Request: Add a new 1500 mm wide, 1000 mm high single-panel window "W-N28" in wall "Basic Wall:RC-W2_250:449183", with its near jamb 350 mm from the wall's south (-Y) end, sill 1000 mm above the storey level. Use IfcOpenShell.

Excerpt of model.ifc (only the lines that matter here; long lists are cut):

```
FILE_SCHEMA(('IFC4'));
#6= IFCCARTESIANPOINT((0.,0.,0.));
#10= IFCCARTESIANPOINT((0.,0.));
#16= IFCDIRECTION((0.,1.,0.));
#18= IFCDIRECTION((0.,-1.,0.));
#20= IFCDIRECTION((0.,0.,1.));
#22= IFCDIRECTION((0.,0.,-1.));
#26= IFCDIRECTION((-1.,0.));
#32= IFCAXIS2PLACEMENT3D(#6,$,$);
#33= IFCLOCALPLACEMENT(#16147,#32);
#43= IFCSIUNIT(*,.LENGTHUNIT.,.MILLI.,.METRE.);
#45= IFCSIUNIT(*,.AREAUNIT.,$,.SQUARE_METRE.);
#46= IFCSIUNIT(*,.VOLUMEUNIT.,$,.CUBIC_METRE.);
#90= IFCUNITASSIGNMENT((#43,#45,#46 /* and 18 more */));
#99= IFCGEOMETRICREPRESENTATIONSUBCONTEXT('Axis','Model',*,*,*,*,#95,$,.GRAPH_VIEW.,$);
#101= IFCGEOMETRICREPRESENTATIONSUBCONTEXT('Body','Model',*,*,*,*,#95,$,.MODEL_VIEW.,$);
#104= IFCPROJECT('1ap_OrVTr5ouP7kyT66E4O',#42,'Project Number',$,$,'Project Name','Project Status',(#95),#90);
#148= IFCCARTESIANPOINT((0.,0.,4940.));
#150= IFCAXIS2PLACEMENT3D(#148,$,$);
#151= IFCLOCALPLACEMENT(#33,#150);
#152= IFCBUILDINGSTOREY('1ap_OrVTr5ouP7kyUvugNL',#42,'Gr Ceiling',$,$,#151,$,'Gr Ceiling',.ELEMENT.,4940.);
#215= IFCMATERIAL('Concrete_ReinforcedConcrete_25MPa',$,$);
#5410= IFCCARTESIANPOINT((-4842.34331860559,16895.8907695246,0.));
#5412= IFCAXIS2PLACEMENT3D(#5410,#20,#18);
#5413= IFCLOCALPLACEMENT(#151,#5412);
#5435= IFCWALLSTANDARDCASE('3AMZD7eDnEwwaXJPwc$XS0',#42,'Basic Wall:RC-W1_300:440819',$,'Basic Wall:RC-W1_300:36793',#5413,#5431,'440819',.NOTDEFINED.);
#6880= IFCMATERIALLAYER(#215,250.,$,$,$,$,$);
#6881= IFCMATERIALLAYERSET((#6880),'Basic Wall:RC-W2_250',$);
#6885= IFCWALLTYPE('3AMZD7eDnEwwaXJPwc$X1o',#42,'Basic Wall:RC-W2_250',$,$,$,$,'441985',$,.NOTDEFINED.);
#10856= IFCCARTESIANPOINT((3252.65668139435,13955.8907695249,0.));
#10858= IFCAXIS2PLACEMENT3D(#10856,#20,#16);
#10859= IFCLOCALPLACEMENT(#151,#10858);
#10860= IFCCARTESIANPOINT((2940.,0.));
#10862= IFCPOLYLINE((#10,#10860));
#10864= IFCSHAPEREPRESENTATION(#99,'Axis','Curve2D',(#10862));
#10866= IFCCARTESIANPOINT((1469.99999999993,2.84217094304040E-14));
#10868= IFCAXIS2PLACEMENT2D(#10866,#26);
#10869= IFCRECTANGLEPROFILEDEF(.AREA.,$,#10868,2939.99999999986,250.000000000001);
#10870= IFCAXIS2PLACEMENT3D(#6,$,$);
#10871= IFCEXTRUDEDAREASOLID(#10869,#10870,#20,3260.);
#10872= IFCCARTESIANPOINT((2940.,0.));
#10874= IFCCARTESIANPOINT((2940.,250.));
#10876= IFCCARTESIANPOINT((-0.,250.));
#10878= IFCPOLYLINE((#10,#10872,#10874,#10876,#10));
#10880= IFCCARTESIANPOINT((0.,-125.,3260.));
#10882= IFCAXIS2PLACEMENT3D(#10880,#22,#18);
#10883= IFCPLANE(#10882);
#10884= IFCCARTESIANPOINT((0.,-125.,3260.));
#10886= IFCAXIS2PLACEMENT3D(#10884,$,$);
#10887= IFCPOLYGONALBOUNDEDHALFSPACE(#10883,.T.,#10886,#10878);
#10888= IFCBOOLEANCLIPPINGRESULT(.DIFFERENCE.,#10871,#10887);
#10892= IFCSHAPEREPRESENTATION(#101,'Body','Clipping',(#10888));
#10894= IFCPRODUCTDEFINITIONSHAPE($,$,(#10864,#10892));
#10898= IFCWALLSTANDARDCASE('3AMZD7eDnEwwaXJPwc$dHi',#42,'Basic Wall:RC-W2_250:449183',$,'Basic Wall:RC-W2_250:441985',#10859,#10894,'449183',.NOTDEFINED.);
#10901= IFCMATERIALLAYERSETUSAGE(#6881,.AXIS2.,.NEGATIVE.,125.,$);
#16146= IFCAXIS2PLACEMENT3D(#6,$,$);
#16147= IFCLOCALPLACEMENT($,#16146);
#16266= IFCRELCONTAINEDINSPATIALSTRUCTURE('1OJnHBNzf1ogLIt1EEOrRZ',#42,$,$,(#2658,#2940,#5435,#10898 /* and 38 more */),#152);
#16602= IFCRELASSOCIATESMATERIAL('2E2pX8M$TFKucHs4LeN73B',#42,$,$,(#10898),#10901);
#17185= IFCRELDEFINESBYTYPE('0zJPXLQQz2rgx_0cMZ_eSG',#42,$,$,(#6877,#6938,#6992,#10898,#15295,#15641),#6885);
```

```python
import numpy as np
import ifcopenshell
import ifcopenshell.api.feature
import ifcopenshell.api.geometry
import ifcopenshell.api.root
import ifcopenshell.api.spatial
import ifcopenshell.geom
import ifcopenshell.util.element
import ifcopenshell.util.placement
import ifcopenshell.util.representation
import ifcopenshell.util.shape
import ifcopenshell.util.unit

model = ifcopenshell.open("model.ifc")
unit_scale = ifcopenshell.util.unit.calculate_unit_scale(model)
settings = ifcopenshell.geom.settings()


def volume(element):
    """Net volume in cubic metres, openings subtracted."""
    shape = ifcopenshell.geom.create_shape(settings, element)
    return ifcopenshell.util.shape.get_volume(shape.geometry)


wall = model.by_guid("3AMZD7eDnEwwaXJPwc$dHi")
storey = ifcopenshell.util.element.get_container(wall, ifc_class="IfcBuildingStorey")
context = ifcopenshell.util.representation.get_context(model, "Model", "Body", "MODEL_VIEW")
before = volume(wall)

width, height, from_end, sill = 1.5, 1, 0.35, 1  # metres

# The wall runs along its own X axis, and the end named is its -X end.
wall_shape = ifcopenshell.geom.create_shape(settings, wall)
x, y, z = ifcopenshell.util.shape.get_vertices(wall_shape.geometry).T
start = x.min() + from_end
face, thickness = float(y.min()), float(y.max() - y.min())
wall_matrix = ifcopenshell.util.placement.get_local_placement(wall.ObjectPlacement)
level = ifcopenshell.util.placement.get_local_placement(storey.ObjectPlacement)[2, 3]


def in_wall(x, y):
    """Placement at x, y metres in the wall's axes, at sill height."""
    matrix = wall_matrix.copy()
    matrix[:, 3] = wall_matrix @ np.array([x / unit_scale, y / unit_scale, 0.0, 1.0])
    matrix[2, 3] = level + sill / unit_scale
    return matrix


# Opening: a box that overshoots both wall faces by 50 mm.
opening = ifcopenshell.api.root.create_entity(model, ifc_class="IfcOpeningElement", predefined_type="OPENING")
box = ifcopenshell.api.geometry.add_wall_representation(
    model, context=context, length=width, height=height, thickness=thickness + 0.1
)
ifcopenshell.api.geometry.assign_representation(model, product=opening, representation=box)
ifcopenshell.api.geometry.edit_object_placement(model, product=opening, matrix=in_wall(start, face - 0.05), is_si=False)
ifcopenshell.api.feature.add_feature(model, feature=opening, element=wall)

window = ifcopenshell.api.root.create_entity(model, ifc_class="IfcWindow", name="W-N28", predefined_type="WINDOW")
window.OverallWidth, window.OverallHeight = width / unit_scale, height / unit_scale
window.PartitioningType = "SINGLE_PANEL"
body = ifcopenshell.api.geometry.add_window_representation(
    model,
    context=context,
    overall_width=window.OverallWidth,
    overall_height=window.OverallHeight,
    partition_type="SINGLE_PANEL",
)
ifcopenshell.api.geometry.assign_representation(model, product=window, representation=body)
ifcopenshell.api.spatial.assign_container(model, products=[window], relating_structure=storey)
ifcopenshell.api.feature.add_filling(model, opening=opening, element=window)

# Centre the window in the wall's thickness.
ifcopenshell.api.geometry.edit_object_placement(model, product=window, matrix=in_wall(start, face), is_si=False)
window_shape = ifcopenshell.geom.create_shape(settings, window)
depth = ifcopenshell.util.shape.get_vertices(window_shape.geometry)[:, 1]
offset = face + thickness / 2 - (depth.min() + depth.max()) / 2
ifcopenshell.api.geometry.edit_object_placement(model, product=window, matrix=in_wall(start, offset), is_si=False)

after = volume(wall)

print(f"wall volume {before:.3f} -> {after:.3f} m3")

model.write("model_v2.ifc")
```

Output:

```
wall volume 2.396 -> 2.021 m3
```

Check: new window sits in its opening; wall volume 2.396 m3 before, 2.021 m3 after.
